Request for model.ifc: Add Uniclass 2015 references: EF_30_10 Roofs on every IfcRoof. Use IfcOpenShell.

First a look at what the model holds.

```python
import ifcopenshell

model = ifcopenshell.open("model.ifc")
print(model.schema)
print("classifications:", [c.Name for c in model.by_type("IfcClassification")])
for ifc_class in ("IfcDoor", "IfcRoof", "IfcStair", "IfcWall", "IfcWindow"):
    print(ifc_class, len(model.by_type(ifc_class)))
```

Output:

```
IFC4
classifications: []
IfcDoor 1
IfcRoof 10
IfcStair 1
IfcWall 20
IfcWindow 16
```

```python
import ifcopenshell
import ifcopenshell.api.classification

model = ifcopenshell.open("model.ifc")

system = ifcopenshell.api.classification.add_classification(model, classification="Uniclass 2015")

codes = {
    "IfcRoof": ("EF_30_10", "Roofs"),
}
for ifc_class, (code, name) in codes.items():
    products = model.by_type(ifc_class)
    ifcopenshell.api.classification.add_reference(
        model, products=products, classification=system, identification=code, name=name
    )
    print(code, len(products))

model.write("model_v2.ifc")
```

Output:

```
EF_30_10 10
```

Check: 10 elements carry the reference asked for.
